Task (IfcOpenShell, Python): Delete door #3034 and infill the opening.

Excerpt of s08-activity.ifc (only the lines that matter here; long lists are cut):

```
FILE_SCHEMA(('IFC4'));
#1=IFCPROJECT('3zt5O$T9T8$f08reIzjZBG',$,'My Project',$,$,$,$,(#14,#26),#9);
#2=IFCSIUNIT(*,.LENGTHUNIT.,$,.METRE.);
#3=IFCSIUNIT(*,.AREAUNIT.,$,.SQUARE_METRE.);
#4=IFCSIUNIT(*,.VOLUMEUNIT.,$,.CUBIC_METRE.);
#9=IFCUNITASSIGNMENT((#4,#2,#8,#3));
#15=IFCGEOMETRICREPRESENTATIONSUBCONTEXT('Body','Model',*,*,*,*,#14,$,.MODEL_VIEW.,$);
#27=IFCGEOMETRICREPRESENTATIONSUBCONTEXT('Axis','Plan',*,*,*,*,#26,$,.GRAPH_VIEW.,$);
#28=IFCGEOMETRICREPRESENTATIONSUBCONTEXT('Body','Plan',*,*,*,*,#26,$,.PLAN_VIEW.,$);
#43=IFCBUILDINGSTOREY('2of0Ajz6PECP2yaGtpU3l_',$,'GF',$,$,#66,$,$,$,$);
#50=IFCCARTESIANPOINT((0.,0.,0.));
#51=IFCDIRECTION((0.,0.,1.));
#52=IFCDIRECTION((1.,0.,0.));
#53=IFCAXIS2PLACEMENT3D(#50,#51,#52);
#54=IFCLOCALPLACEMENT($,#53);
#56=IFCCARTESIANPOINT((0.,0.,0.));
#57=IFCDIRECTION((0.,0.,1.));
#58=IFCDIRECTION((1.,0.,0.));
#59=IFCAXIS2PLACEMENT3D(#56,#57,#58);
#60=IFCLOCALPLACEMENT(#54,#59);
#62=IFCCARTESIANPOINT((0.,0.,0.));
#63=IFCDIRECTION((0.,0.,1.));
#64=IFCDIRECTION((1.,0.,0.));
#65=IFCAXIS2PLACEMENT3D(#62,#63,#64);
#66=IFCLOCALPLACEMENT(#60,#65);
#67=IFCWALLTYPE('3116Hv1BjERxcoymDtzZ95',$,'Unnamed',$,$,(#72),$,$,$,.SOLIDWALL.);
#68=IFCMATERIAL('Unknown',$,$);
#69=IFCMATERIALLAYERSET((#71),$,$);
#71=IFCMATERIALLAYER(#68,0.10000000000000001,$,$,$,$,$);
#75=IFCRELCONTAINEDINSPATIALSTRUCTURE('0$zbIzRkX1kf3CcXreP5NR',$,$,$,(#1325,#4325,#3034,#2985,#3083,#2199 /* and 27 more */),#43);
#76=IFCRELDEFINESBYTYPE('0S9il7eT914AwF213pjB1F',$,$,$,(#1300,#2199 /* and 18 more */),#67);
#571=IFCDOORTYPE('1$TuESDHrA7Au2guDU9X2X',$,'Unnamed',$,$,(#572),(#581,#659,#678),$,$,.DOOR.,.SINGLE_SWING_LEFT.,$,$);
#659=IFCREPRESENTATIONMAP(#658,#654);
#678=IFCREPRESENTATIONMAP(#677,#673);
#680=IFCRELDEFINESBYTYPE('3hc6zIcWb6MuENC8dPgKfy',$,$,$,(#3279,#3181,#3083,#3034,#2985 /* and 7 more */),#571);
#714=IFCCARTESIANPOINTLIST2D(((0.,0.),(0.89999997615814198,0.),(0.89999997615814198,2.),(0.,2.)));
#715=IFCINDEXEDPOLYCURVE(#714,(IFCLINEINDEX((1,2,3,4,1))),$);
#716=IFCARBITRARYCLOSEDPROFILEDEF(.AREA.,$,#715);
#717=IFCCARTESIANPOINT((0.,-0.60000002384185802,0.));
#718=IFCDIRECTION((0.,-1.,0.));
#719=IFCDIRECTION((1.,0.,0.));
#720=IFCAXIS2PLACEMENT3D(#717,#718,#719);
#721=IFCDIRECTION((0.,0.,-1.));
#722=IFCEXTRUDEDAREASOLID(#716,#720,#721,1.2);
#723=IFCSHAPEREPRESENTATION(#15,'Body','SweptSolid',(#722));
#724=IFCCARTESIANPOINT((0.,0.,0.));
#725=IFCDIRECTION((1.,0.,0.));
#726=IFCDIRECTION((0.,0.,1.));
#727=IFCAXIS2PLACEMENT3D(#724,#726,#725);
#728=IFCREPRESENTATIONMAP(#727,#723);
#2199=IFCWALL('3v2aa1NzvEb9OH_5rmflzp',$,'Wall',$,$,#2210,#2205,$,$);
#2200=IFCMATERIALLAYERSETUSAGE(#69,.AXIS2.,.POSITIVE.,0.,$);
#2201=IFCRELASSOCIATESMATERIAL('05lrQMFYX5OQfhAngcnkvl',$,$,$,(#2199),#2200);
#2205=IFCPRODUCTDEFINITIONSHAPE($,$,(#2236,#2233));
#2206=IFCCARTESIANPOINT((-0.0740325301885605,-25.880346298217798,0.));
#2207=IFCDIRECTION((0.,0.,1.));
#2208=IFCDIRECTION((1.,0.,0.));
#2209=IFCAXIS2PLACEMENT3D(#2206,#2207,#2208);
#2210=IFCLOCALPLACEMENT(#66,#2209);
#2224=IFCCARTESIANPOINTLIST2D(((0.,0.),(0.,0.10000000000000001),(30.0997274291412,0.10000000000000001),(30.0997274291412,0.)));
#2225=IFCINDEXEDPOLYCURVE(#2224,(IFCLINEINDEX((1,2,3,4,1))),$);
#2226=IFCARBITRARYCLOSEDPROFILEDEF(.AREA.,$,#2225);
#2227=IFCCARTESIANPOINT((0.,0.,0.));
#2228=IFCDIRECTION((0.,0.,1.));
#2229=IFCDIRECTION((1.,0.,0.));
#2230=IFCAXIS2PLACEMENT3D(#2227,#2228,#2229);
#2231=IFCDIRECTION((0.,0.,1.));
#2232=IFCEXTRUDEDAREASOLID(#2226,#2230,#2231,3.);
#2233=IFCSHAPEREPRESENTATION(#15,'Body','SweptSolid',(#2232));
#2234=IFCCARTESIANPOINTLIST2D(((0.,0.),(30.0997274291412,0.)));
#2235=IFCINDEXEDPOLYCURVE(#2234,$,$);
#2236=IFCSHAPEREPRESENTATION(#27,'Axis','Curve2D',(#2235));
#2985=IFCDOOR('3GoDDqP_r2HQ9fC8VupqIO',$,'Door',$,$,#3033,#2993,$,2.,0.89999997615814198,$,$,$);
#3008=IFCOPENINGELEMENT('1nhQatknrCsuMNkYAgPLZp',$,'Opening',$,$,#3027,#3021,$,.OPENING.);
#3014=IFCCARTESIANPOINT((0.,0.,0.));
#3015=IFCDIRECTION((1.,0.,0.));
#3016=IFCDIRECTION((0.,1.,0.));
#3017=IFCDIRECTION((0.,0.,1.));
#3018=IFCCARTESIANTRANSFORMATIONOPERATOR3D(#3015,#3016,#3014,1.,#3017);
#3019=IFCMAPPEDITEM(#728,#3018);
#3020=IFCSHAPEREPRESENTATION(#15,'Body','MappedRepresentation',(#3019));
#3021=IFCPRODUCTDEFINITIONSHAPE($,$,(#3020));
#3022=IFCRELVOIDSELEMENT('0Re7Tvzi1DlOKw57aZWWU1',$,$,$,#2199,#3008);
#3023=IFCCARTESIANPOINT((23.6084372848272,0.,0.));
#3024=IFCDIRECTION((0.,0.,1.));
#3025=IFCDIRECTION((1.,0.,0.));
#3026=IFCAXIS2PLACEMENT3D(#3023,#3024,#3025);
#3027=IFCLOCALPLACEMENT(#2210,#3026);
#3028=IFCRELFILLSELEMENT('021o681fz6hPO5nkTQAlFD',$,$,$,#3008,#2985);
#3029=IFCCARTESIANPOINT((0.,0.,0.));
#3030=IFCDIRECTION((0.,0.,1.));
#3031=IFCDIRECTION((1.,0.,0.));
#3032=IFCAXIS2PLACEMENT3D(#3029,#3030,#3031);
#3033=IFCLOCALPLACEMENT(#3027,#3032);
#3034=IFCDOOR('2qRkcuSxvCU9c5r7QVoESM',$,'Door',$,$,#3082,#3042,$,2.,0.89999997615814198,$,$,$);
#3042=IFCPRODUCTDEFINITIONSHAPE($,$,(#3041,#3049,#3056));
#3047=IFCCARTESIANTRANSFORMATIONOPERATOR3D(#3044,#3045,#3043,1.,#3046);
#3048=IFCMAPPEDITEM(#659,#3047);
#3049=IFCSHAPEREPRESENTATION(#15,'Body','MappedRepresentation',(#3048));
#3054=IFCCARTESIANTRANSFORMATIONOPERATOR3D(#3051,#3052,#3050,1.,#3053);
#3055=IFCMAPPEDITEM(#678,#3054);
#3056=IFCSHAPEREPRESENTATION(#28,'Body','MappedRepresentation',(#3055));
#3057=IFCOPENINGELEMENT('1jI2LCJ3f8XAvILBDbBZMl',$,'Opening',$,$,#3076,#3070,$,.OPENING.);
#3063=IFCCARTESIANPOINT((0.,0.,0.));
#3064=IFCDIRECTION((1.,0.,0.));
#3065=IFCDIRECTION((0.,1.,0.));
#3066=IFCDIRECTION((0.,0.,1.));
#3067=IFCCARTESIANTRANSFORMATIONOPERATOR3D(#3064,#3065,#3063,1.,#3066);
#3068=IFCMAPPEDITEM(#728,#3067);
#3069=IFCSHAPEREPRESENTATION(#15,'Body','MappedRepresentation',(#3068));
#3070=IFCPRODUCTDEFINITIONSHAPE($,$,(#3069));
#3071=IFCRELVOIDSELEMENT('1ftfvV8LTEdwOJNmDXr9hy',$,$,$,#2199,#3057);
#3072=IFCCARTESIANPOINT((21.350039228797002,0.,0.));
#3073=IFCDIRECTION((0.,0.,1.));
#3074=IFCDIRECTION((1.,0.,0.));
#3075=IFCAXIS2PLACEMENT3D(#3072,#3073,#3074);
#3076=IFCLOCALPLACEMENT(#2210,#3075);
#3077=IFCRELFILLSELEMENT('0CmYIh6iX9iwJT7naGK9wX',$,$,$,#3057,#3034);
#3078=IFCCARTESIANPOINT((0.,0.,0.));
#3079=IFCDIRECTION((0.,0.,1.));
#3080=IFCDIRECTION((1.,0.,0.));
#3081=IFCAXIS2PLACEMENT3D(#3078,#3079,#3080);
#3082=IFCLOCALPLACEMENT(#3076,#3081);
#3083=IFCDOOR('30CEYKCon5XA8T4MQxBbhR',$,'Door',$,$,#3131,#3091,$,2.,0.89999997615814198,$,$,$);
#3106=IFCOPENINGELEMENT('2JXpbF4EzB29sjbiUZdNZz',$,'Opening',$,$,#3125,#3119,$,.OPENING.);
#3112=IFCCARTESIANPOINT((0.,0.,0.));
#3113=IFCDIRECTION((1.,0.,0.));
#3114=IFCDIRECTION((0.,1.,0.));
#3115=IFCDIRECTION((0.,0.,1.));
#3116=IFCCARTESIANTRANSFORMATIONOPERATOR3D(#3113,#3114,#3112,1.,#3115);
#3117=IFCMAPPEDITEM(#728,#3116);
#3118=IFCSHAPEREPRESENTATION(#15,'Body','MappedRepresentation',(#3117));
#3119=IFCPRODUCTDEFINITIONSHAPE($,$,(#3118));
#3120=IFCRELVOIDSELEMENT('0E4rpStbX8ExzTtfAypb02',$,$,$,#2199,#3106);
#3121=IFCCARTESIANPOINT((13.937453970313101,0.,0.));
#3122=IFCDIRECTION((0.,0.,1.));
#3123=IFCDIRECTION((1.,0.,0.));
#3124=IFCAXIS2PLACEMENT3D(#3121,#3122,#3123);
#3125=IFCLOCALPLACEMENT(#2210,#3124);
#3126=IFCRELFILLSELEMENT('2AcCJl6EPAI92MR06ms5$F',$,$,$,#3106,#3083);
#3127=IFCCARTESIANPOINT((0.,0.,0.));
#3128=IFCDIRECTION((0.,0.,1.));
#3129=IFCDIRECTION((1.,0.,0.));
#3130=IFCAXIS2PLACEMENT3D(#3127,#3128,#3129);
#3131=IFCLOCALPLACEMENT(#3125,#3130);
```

```python
import ifcopenshell
import ifcopenshell.api.feature
import ifcopenshell.api.root
import ifcopenshell.geom
import ifcopenshell.util.shape

model = ifcopenshell.open("s08-activity.ifc")
settings = ifcopenshell.geom.settings()


def volume(element):
    """Net volume in cubic metres, openings subtracted."""
    shape = ifcopenshell.geom.create_shape(settings, element)
    return ifcopenshell.util.shape.get_volume(shape.geometry)


door = model.by_guid("2qRkcuSxvCU9c5r7QVoESM")
opening = door.FillsVoids[0].RelatingOpeningElement
wall = opening.VoidsElements[0].RelatingBuildingElement
before = volume(wall)

ifcopenshell.api.root.remove_product(model, product=door)
ifcopenshell.api.feature.remove_feature(model, feature=opening)

after = volume(wall)

print(f"wall volume {before:.3f} -> {after:.3f} m3")

model.write("s08-activity_updated.ifc")
```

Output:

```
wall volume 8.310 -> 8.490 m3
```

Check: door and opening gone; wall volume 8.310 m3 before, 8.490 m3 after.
